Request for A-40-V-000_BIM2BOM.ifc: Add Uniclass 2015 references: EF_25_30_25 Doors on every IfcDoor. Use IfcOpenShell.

First a look at what the model holds.

```python
import ifcopenshell

model = ifcopenshell.open("A-40-V-000_BIM2BOM.ifc")
print(model.schema)
print("classifications:", [c.Name for c in model.by_type("IfcClassification")])
for ifc_class in ("IfcDoor", "IfcRoof", "IfcStair", "IfcWall", "IfcWindow"):
    print(ifc_class, len(model.by_type(ifc_class)))
```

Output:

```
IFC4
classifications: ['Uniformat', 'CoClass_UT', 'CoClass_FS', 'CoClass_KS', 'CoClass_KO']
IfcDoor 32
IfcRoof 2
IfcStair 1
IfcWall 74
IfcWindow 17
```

```python
import ifcopenshell
import ifcopenshell.api.classification

model = ifcopenshell.open("A-40-V-000_BIM2BOM.ifc")

system = ifcopenshell.api.classification.add_classification(model, classification="Uniclass 2015")

codes = {
    "IfcDoor": ("EF_25_30_25", "Doors"),
}
for ifc_class, (code, name) in codes.items():
    products = model.by_type(ifc_class)
    ifcopenshell.api.classification.add_reference(
        model, products=products, classification=system, identification=code, name=name
    )
    print(code, len(products))

model.write("A-40-V-000_BIM2BOM_v2.ifc")
```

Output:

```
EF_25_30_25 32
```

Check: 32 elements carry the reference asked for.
